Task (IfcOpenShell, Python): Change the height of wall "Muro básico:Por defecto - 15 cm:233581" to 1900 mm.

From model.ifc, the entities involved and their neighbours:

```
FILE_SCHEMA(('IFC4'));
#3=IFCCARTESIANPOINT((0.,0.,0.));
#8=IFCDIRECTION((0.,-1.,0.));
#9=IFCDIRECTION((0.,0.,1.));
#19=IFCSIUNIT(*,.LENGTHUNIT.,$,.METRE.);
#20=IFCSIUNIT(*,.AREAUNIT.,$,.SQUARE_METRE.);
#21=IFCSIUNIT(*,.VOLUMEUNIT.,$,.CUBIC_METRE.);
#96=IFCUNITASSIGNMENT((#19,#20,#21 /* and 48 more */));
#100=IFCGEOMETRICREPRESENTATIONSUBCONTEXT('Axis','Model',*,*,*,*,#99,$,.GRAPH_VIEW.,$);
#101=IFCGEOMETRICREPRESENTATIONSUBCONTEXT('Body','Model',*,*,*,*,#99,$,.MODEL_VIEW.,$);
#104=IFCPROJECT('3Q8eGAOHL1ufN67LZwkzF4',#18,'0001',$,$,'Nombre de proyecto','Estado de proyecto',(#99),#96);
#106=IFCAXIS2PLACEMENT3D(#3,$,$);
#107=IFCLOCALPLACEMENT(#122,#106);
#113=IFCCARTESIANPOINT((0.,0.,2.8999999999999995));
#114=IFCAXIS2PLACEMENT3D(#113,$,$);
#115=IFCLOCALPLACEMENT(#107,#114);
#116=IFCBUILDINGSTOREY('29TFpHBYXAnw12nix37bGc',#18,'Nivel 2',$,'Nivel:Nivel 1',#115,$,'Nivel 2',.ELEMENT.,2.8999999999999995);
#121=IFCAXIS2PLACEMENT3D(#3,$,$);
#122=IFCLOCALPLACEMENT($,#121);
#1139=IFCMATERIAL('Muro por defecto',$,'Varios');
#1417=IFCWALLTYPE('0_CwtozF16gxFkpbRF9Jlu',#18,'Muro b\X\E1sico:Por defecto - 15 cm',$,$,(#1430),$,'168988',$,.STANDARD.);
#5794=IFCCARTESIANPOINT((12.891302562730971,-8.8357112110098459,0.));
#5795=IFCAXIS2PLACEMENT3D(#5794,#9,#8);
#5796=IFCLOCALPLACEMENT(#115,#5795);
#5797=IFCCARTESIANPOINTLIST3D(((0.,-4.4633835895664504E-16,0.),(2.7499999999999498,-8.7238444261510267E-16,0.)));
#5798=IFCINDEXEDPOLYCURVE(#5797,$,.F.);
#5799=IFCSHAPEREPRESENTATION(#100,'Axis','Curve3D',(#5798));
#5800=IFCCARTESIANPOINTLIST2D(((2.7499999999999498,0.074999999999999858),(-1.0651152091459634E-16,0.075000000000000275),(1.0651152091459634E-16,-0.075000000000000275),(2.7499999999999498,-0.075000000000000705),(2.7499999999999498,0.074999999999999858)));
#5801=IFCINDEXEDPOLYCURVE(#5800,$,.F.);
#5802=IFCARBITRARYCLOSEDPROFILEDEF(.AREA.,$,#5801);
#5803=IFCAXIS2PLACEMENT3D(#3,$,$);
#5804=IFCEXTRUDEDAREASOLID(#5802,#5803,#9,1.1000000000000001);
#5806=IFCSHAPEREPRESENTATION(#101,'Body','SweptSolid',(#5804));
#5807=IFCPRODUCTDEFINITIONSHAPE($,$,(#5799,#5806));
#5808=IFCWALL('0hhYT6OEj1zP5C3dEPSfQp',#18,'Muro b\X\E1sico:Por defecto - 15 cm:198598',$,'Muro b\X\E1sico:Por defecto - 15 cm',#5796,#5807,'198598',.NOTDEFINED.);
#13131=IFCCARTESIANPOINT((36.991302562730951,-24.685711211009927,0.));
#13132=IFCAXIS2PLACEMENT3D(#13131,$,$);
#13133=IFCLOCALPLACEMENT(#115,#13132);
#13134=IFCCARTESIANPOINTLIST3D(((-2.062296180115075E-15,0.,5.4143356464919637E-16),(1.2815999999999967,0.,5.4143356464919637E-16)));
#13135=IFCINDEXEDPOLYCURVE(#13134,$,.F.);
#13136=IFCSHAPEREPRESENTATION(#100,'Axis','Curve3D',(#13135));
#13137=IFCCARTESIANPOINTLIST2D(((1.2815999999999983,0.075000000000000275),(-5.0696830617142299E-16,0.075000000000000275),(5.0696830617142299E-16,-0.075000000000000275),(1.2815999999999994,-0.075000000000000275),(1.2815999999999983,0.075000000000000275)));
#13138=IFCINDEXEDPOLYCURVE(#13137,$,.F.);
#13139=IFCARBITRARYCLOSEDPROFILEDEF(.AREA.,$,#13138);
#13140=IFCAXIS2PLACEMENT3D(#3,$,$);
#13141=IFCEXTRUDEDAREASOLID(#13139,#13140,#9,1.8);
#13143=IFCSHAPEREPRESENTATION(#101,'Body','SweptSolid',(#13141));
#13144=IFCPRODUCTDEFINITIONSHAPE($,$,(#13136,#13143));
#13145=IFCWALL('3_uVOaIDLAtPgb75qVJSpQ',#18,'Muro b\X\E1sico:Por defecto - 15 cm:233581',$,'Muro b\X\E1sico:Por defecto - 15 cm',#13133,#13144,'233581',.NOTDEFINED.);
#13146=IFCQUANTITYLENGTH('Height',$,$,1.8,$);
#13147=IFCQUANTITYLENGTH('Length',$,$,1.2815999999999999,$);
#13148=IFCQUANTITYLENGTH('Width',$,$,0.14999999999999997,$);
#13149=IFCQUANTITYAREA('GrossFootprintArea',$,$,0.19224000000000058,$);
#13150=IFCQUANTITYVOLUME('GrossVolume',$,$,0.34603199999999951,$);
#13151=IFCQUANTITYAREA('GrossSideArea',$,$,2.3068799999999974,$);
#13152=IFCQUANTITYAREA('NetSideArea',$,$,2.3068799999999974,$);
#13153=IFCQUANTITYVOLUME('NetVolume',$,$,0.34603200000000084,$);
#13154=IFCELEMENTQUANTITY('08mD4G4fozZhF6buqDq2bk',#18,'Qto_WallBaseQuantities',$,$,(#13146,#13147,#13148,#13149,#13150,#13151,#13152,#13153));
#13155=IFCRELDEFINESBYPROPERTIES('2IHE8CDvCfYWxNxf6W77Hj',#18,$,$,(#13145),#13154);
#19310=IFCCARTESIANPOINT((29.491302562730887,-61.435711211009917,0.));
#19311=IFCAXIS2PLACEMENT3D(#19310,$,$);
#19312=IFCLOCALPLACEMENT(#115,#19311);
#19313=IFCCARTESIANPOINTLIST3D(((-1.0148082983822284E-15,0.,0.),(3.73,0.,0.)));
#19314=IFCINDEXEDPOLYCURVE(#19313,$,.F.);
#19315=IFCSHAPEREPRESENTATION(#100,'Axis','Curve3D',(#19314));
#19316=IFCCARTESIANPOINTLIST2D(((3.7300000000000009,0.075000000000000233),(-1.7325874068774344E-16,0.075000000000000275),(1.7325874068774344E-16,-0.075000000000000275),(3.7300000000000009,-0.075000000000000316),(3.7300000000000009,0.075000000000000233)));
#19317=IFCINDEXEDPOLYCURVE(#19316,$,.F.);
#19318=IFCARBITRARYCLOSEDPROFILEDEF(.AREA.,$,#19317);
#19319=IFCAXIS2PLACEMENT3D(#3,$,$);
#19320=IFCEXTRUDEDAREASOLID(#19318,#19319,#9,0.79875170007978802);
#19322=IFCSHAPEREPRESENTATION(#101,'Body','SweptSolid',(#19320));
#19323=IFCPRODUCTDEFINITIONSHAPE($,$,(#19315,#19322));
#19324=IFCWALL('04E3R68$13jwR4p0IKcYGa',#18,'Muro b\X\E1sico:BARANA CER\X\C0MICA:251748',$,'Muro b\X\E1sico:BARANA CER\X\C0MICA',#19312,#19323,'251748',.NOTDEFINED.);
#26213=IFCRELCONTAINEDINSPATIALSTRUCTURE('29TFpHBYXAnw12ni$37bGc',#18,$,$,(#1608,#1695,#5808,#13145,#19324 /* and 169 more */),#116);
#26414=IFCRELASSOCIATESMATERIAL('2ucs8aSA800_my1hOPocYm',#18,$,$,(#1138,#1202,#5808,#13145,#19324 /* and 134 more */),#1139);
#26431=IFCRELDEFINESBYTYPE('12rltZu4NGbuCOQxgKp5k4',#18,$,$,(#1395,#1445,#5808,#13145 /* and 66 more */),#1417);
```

```python
import ifcopenshell
import ifcopenshell.api.pset
import ifcopenshell.geom
import ifcopenshell.util.element
import ifcopenshell.util.representation
import ifcopenshell.util.shape
import ifcopenshell.util.unit

model = ifcopenshell.open("model.ifc")
unit_scale = ifcopenshell.util.unit.calculate_unit_scale(model)
area_scale = ifcopenshell.util.unit.calculate_unit_scale(model, "AREAUNIT")
volume_scale = ifcopenshell.util.unit.calculate_unit_scale(model, "VOLUMEUNIT")
settings = ifcopenshell.geom.settings()


def volume(element):
    """Net volume in cubic metres, openings subtracted."""
    shape = ifcopenshell.geom.create_shape(settings, element)
    return ifcopenshell.util.shape.get_volume(shape.geometry)


wall = model.by_guid("3_uVOaIDLAtPgb75qVJSpQ")
before = volume(wall)

body = ifcopenshell.util.representation.get_representation(wall, "Model", "Body")
solid = body.Items[0]
old_height = solid.Depth
solid.Depth = 1.9 / unit_scale
after = volume(wall)
thickness = 0.15  # wall thickness in metres

# Update the stored height, areas and volumes.
qto = model.by_id(ifcopenshell.util.element.get_pset(wall, "Qto_WallBaseQuantities", should_inherit=False)["id"])
ifcopenshell.api.pset.edit_qto(model, qto=qto, properties={
    "Height": solid.Depth,
    "GrossVolume": ifcopenshell.util.element.get_pset(wall, "Qto_WallBaseQuantities", "GrossVolume") * solid.Depth / old_height,
    "GrossSideArea": ifcopenshell.util.element.get_pset(wall, "Qto_WallBaseQuantities", "GrossSideArea") * solid.Depth / old_height,
    "NetSideArea": after / thickness / area_scale,
    "NetVolume": after / volume_scale,
})

print(f"height {old_height:g} -> {solid.Depth:g}, volume {before:.3f} -> {after:.3f} m3")

model.write("model_updated.ifc")
```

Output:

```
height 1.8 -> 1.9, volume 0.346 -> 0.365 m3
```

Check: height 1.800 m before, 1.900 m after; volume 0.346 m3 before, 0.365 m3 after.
